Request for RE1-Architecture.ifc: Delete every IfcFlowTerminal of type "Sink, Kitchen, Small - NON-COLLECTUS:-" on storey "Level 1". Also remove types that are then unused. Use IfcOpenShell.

First a look at what the model holds.

```python
import ifcopenshell
import ifcopenshell.util.element

model = ifcopenshell.open("RE1-Architecture.ifc")
print(model.schema)
storey = next(s for s in model.by_type("IfcBuildingStorey") if s.Name == "Level 1")
terminals = [e for e in ifcopenshell.util.element.get_decomposition(storey) if e.is_a("IfcFlowTerminal")]
seen = {}
for e in terminals:
    element_type = ifcopenshell.util.element.get_type(e)
    name = element_type.Name if element_type not in (None, e) else None
    seen[name] = seen.get(name, 0) + 1
for name, count in sorted(seen.items(), key=str):
    print(count, "x", name)
```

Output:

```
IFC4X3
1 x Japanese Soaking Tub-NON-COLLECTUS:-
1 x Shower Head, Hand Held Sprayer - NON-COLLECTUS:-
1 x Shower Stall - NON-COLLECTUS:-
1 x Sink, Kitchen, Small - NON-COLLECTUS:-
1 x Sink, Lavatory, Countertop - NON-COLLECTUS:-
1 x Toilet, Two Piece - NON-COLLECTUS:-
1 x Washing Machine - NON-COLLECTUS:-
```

```python
import ifcopenshell
import ifcopenshell.api.root
import ifcopenshell.util.element

model = ifcopenshell.open("RE1-Architecture.ifc")

storey = next(s for s in model.by_type("IfcBuildingStorey") if s.Name == "Level 1")
terminals = [e for e in ifcopenshell.util.element.get_decomposition(storey) if e.is_a("IfcFlowTerminal")]
targets = [e for e in terminals if (t := ifcopenshell.util.element.get_type(e)) not in (None, e) and t.Name == "Sink, Kitchen, Small - NON-COLLECTUS:-"]
types = {ifcopenshell.util.element.get_type(e) for e in targets} - {None, *targets}

for e in targets:
    ifcopenshell.api.root.remove_product(model, product=e)
print(len(targets), "removed")

unused = [t for t in types if not ifcopenshell.util.element.get_types(t)]
for t in unused:
    ifcopenshell.api.root.remove_product(model, product=t)
print(len(unused), "unused types removed")

model.write("RE1-Architecture_v2.ifc")
```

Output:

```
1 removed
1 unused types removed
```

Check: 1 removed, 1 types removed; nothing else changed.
